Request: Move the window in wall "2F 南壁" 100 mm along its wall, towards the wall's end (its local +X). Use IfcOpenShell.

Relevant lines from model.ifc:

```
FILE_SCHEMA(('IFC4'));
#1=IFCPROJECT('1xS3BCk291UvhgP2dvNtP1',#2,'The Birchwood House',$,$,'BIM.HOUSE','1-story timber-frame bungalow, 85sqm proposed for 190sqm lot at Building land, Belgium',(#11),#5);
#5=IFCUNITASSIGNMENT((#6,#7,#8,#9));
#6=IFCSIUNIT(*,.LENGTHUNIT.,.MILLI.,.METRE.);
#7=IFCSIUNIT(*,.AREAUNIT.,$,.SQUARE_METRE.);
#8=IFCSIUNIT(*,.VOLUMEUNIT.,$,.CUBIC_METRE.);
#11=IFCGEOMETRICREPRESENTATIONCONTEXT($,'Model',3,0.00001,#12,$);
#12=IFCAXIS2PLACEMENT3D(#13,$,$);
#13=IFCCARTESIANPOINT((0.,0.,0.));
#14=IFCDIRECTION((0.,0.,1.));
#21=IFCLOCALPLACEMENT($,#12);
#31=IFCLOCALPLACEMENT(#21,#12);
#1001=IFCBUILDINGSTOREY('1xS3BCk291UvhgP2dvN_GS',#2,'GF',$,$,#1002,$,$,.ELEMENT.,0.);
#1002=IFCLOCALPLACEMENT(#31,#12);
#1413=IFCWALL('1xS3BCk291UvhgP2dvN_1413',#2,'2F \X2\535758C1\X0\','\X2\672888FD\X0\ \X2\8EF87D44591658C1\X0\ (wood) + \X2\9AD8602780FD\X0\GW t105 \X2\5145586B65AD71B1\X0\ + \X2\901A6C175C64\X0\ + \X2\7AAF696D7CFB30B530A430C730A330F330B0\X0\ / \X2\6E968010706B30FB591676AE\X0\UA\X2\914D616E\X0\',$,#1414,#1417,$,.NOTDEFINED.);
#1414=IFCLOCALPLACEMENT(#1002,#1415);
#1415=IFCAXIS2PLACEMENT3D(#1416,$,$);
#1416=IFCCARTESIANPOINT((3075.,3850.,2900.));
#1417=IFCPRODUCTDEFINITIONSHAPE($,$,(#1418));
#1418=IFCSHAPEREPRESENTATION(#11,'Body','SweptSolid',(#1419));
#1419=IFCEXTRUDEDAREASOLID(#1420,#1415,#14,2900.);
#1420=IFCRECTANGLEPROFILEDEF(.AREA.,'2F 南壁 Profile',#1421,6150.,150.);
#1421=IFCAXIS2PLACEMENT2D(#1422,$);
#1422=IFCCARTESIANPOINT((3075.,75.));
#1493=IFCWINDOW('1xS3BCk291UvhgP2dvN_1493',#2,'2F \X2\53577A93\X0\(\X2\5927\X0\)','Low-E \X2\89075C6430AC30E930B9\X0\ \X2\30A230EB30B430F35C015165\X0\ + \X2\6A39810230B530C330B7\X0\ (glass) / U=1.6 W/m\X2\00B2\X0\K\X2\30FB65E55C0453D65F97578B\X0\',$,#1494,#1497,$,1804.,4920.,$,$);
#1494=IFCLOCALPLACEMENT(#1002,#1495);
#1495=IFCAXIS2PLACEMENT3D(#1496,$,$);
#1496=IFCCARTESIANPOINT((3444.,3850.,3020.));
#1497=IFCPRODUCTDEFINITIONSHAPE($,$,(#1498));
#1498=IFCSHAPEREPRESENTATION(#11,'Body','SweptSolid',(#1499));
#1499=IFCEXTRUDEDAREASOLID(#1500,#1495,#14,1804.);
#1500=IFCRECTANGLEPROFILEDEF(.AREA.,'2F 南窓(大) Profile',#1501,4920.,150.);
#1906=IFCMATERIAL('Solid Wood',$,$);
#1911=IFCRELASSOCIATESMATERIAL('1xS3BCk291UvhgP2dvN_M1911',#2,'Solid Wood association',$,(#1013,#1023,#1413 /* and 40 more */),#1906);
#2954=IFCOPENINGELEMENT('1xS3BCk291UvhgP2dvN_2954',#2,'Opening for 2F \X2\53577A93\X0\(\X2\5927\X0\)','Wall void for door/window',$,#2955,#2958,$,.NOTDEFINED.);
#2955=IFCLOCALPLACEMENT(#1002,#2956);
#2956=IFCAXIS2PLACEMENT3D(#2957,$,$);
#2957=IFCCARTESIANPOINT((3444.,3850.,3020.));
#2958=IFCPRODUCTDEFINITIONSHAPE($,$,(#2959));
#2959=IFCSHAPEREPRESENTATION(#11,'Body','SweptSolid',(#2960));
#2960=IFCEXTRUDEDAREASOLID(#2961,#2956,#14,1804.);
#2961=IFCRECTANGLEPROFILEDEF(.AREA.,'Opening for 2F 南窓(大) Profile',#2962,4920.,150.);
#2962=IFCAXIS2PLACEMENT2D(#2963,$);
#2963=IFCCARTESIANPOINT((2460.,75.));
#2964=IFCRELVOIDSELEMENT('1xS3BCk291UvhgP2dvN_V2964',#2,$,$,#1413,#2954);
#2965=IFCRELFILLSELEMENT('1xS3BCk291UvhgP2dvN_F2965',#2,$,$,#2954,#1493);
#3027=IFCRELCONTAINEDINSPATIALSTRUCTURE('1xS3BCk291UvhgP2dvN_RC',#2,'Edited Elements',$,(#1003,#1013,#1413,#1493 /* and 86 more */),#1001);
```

```python
import ifcopenshell
import ifcopenshell.api.geometry
import ifcopenshell.util.placement
import ifcopenshell.util.unit

model = ifcopenshell.open("model.ifc")
unit_scale = ifcopenshell.util.unit.calculate_unit_scale(model)

window = model.by_id(1493)
opening = window.FillsVoids[0].RelatingOpeningElement
wall = opening.VoidsElements[0].RelatingBuildingElement

wall_matrix = ifcopenshell.util.placement.get_local_placement(wall.ObjectPlacement)
shift = wall_matrix[:3, 0] * 0.1 / unit_scale
before = ifcopenshell.util.placement.get_local_placement(window.ObjectPlacement)[:3, 3].copy()

# The window is not placed relative to its opening, so move both.
for product in (opening, window):
    matrix = ifcopenshell.util.placement.get_local_placement(product.ObjectPlacement)
    matrix[:3, 3] += shift
    ifcopenshell.api.geometry.edit_object_placement(model, product=product, matrix=matrix, is_si=False)

after = ifcopenshell.util.placement.get_local_placement(window.ObjectPlacement)[:3, 3]
print("window moved by", (after - before).round(3) + 0.0)

model.write("model_updated.ifc")
```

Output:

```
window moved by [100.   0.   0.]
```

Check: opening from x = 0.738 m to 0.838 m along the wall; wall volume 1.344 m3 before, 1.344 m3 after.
